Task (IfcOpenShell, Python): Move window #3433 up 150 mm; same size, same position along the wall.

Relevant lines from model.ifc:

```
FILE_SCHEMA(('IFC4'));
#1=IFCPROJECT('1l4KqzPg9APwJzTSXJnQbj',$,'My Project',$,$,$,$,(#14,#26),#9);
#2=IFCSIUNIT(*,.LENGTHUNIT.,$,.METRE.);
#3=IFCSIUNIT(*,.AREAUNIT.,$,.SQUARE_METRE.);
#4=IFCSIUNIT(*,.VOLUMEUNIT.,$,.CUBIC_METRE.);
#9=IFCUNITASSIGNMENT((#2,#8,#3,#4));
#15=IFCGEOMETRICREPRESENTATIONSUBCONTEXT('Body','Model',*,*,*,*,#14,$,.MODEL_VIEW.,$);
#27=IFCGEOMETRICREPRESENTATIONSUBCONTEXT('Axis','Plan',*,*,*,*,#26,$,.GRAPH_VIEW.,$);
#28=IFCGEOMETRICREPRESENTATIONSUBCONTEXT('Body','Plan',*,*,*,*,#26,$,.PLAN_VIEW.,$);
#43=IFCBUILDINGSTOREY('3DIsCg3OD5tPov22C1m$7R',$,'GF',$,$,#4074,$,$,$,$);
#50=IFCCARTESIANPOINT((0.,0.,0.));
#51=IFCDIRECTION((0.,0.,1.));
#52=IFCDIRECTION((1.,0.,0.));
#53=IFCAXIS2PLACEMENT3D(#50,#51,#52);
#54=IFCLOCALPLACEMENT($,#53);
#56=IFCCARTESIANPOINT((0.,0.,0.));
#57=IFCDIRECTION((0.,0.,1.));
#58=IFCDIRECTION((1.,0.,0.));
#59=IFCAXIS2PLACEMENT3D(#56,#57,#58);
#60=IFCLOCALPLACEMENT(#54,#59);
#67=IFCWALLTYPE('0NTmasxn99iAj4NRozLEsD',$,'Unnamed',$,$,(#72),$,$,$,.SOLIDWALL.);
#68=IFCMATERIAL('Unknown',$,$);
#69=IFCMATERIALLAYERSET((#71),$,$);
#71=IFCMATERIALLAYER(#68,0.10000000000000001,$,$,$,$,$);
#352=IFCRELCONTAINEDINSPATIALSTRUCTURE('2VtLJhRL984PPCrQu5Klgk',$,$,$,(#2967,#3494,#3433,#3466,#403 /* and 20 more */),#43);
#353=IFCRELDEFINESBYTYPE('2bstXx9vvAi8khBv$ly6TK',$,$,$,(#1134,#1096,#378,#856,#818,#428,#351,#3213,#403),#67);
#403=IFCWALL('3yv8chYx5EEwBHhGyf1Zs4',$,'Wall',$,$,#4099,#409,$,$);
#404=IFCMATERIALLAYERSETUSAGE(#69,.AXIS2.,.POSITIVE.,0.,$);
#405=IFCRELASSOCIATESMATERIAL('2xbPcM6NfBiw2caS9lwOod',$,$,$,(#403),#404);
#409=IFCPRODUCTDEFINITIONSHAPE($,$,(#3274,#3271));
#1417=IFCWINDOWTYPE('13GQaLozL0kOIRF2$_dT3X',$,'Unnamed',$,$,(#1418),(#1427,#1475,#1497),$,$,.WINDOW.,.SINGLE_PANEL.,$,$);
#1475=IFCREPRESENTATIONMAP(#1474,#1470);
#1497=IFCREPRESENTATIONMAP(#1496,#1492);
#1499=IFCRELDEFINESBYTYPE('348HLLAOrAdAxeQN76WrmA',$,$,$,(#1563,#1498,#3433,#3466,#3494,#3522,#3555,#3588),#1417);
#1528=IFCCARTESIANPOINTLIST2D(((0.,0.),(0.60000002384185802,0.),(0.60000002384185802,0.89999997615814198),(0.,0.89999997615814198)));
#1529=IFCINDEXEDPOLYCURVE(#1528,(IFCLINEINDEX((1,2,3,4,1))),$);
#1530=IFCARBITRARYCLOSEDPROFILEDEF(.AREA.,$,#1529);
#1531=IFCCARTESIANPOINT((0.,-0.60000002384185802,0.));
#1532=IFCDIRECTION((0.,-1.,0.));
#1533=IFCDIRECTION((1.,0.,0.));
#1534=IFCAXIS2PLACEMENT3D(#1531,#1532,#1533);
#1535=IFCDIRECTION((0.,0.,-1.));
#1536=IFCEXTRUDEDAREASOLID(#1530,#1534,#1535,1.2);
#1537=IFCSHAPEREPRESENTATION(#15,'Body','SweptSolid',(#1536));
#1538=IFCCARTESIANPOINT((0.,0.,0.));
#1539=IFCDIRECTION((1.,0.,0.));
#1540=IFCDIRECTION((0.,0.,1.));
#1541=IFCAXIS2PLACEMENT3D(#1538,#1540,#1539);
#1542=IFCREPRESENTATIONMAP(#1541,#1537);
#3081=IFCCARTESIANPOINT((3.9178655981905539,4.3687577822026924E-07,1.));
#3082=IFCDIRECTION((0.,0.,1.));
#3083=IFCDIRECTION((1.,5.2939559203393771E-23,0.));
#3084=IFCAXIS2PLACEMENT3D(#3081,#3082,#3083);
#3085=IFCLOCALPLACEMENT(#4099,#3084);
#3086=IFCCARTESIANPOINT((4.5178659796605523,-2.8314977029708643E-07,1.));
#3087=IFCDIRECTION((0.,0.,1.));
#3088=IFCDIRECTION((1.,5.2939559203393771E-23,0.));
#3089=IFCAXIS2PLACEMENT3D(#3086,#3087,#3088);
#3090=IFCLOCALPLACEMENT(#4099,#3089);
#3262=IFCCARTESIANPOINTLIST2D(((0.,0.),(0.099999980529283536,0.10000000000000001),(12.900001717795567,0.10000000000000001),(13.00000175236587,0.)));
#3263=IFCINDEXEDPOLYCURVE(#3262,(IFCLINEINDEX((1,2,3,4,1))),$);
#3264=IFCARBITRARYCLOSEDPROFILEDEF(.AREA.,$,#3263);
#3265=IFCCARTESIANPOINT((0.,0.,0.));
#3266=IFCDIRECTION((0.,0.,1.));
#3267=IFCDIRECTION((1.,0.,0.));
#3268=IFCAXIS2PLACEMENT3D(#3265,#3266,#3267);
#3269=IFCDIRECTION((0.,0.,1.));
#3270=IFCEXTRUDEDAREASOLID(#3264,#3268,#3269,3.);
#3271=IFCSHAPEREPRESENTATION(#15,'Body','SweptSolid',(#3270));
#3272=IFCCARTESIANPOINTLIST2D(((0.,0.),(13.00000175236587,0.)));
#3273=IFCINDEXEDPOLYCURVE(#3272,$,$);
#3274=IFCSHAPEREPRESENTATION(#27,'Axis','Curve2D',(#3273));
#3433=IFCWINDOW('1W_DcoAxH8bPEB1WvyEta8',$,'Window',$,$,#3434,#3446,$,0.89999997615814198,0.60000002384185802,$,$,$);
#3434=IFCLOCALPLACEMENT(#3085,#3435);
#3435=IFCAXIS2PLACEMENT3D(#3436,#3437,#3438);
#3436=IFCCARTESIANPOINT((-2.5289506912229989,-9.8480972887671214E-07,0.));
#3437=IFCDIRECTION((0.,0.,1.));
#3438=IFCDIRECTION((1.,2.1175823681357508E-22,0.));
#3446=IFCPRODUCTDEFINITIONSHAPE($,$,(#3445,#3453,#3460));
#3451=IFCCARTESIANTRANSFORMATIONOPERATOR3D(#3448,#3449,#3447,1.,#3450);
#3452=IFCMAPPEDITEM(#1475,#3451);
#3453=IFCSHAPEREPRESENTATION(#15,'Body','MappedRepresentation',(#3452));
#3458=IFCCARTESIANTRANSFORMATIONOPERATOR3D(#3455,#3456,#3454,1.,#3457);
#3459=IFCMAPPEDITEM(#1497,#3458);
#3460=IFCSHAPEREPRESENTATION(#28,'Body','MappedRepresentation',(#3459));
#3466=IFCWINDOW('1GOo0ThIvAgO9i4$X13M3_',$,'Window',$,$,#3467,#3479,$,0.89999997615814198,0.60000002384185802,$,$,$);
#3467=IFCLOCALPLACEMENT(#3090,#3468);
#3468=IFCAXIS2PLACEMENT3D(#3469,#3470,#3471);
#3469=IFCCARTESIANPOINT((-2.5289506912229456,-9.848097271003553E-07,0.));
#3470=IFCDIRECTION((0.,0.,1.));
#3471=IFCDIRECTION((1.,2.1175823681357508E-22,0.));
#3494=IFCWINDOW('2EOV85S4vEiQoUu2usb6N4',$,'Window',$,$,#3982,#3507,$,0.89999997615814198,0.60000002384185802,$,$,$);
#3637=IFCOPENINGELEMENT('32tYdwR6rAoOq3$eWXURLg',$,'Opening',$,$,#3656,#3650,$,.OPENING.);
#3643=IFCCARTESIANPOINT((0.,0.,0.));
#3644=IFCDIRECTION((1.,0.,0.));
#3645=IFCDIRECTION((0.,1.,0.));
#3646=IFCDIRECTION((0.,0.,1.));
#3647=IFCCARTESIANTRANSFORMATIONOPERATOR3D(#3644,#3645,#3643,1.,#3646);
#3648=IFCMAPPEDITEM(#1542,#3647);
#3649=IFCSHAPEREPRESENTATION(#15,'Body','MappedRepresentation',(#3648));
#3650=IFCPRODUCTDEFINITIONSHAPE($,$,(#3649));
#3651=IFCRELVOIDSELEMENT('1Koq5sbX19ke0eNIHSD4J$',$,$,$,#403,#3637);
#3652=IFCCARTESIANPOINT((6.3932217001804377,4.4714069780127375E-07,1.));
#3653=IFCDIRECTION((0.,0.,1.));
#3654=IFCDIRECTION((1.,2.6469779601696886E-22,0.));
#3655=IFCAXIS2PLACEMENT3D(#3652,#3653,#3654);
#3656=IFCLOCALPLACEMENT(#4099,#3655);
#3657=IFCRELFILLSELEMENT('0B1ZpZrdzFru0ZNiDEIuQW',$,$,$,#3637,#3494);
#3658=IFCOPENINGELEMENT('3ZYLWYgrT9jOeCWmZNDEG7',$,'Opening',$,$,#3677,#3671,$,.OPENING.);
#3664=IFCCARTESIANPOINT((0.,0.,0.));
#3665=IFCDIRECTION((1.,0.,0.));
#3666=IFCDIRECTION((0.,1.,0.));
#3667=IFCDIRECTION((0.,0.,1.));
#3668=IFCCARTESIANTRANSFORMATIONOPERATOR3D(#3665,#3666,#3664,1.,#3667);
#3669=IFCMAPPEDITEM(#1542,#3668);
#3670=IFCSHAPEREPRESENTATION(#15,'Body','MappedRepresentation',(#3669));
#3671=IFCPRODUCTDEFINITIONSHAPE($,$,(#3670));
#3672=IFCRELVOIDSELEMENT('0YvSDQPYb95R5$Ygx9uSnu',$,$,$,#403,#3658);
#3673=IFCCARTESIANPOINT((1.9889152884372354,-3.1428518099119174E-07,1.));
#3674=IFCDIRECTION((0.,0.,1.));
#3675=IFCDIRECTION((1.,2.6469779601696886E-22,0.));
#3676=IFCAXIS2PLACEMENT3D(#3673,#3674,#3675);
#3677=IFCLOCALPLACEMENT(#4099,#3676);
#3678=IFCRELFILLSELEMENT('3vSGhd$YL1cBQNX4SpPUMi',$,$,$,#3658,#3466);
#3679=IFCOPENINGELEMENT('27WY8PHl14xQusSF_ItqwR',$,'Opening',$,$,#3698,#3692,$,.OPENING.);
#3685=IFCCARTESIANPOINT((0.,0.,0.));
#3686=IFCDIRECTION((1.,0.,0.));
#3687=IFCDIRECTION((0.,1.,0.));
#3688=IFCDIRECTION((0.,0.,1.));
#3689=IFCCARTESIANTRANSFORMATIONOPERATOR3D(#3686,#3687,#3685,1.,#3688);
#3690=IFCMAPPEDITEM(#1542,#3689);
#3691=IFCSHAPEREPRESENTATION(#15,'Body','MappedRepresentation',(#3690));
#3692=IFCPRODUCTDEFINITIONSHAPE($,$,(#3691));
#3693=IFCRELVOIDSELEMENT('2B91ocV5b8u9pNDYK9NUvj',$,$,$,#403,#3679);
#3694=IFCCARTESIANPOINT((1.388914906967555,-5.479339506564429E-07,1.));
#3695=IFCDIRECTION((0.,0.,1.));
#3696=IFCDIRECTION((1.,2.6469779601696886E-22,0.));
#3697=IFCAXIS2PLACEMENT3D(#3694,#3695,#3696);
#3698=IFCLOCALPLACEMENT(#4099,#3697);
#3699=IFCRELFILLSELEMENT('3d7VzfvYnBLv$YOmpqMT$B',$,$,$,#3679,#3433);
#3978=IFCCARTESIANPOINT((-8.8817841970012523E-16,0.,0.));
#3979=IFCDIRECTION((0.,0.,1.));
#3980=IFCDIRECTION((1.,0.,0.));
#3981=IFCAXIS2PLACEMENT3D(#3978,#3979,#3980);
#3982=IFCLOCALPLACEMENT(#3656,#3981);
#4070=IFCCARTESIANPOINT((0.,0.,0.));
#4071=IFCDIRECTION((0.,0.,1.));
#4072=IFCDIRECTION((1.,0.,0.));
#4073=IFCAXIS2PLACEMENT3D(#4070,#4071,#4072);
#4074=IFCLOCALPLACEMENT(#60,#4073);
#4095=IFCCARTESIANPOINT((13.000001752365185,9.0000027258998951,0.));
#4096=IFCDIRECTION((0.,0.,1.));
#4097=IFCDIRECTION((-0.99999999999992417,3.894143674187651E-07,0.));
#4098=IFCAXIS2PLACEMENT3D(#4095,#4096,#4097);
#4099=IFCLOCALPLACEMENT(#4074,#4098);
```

```python
import numpy as np
import ifcopenshell
import ifcopenshell.api.geometry
import ifcopenshell.util.placement
import ifcopenshell.util.unit

model = ifcopenshell.open("model.ifc")
unit_scale = ifcopenshell.util.unit.calculate_unit_scale(model)

window = model.by_id(3433)
opening = window.FillsVoids[0].RelatingOpeningElement
dz = 0.15 / unit_scale

shift = np.array([0.0, 0.0, dz])
# The window is not placed relative to its opening, so move both.
for product in (opening, window):
    matrix = ifcopenshell.util.placement.get_local_placement(product.ObjectPlacement)
    matrix[:3, 3] += shift
    ifcopenshell.api.geometry.edit_object_placement(model, product=product, matrix=matrix, is_si=False)

print(f"moved by {dz * unit_scale:+.3f} m")

model.write("model_updated.ifc")
```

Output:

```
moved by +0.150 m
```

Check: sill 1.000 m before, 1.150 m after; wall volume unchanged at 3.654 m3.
